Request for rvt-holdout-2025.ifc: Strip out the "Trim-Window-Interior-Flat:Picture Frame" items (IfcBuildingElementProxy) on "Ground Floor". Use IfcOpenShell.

First a look at what the model holds.

```python
import ifcopenshell
import ifcopenshell.util.element

model = ifcopenshell.open("rvt-holdout-2025.ifc")
print(model.schema)
storey = next(s for s in model.by_type("IfcBuildingStorey") if s.Name == "Ground Floor")
proxies = [e for e in ifcopenshell.util.element.get_decomposition(storey) if e.is_a("IfcBuildingElementProxy")]
seen = {}
for e in proxies:
    element_type = ifcopenshell.util.element.get_type(e)
    name = element_type.Name if element_type not in (None, e) else None
    seen[name] = seen.get(name, 0) + 1
for name, count in sorted(seen.items(), key=str):
    print(count, "x", name)
```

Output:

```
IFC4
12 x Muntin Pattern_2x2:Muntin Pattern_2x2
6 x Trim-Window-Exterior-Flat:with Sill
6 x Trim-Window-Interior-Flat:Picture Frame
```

```python
import ifcopenshell
import ifcopenshell.api.root
import ifcopenshell.util.element

model = ifcopenshell.open("rvt-holdout-2025.ifc")

storey = next(s for s in model.by_type("IfcBuildingStorey") if s.Name == "Ground Floor")
proxies = [e for e in ifcopenshell.util.element.get_decomposition(storey) if e.is_a("IfcBuildingElementProxy")]
targets = [e for e in proxies if (t := ifcopenshell.util.element.get_type(e)) not in (None, e) and t.Name == "Trim-Window-Interior-Flat:Picture Frame"]

for e in targets:
    ifcopenshell.api.root.remove_product(model, product=e)
print(len(targets), "removed")

model.write("rvt-holdout-2025_edited.ifc")
```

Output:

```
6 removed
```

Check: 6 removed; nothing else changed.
